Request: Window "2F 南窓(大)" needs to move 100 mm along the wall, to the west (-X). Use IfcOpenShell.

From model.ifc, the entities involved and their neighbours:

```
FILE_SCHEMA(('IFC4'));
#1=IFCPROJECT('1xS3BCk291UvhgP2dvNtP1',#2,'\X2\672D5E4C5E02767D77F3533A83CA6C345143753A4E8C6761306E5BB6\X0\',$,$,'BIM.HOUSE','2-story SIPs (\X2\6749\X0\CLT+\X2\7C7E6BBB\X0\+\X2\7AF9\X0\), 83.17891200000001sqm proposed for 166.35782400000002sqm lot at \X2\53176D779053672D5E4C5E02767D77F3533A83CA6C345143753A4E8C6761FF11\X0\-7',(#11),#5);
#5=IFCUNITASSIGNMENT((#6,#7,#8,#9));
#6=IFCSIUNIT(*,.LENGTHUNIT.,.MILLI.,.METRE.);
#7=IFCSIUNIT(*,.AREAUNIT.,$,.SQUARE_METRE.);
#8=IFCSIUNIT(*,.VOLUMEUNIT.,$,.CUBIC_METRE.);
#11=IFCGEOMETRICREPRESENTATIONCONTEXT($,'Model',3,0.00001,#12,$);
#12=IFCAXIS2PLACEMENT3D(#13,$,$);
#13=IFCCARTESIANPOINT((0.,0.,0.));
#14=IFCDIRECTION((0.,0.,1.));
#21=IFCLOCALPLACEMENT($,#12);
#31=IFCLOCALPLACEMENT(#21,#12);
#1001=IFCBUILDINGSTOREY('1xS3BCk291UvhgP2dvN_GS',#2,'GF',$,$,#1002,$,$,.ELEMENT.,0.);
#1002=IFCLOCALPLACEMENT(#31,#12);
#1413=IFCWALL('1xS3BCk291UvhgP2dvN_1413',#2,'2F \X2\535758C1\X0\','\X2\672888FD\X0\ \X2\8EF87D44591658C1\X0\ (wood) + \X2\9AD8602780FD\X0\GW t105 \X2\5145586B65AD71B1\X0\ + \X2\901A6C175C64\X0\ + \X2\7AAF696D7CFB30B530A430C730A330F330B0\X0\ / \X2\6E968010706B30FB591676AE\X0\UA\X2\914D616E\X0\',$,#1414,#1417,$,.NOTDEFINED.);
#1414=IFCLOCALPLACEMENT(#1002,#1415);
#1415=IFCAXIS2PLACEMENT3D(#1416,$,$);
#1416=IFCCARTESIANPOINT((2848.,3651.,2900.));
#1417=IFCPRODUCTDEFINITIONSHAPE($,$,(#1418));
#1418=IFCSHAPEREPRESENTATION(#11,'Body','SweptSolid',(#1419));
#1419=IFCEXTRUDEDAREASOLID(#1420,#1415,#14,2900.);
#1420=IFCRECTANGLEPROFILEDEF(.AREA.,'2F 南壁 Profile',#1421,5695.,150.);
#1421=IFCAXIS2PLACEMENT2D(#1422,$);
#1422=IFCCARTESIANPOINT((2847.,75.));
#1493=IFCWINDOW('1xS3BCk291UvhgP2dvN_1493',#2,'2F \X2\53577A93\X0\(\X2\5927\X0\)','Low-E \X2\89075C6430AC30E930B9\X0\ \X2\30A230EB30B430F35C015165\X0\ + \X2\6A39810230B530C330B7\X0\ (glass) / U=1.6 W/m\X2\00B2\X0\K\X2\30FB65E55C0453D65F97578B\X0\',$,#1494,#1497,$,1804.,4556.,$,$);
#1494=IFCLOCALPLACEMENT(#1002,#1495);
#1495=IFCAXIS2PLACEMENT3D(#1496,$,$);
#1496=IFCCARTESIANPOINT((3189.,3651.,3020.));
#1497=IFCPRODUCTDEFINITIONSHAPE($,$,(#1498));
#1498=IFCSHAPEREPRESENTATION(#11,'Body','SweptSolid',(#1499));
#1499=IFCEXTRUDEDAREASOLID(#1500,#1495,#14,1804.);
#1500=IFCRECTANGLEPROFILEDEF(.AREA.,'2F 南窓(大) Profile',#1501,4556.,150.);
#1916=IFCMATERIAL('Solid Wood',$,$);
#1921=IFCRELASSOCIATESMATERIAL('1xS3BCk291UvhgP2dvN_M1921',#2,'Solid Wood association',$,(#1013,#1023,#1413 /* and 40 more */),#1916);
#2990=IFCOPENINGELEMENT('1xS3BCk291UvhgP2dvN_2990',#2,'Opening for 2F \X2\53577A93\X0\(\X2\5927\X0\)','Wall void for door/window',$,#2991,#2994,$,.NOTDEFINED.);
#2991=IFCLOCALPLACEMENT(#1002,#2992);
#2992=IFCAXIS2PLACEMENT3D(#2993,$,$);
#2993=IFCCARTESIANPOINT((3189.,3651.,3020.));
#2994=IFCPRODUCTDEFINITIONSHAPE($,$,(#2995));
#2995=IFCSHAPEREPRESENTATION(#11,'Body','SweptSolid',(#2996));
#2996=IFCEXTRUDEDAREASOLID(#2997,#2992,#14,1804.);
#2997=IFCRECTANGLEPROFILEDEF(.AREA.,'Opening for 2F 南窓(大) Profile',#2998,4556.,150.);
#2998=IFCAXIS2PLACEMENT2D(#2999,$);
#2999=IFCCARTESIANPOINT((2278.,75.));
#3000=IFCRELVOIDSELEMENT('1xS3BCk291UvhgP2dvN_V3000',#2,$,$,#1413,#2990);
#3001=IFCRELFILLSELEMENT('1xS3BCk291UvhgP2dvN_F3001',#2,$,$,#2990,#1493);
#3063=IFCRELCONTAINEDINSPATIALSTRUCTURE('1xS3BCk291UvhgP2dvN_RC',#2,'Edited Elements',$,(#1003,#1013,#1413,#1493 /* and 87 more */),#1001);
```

```python
import ifcopenshell
import ifcopenshell.api.geometry
import ifcopenshell.util.placement

model = ifcopenshell.open("model.ifc")

window = model.by_guid("1xS3BCk291UvhgP2dvN_1493")
opening = window.FillsVoids[0].RelatingOpeningElement
wall = opening.VoidsElements[0].RelatingBuildingElement

wall_matrix = ifcopenshell.util.placement.get_local_placement(wall.ObjectPlacement)
shift = wall_matrix[:3, 0] * -100.0
before = ifcopenshell.util.placement.get_local_placement(window.ObjectPlacement)[:3, 3].copy()

# The window is not placed relative to its opening, so move both.
for product in (opening, window):
    matrix = ifcopenshell.util.placement.get_local_placement(product.ObjectPlacement)
    matrix[:3, 3] += shift
    ifcopenshell.api.geometry.edit_object_placement(model, product=product, matrix=matrix, is_si=False)

after = ifcopenshell.util.placement.get_local_placement(window.ObjectPlacement)[:3, 3]
print("window moved by", (after - before).round(3) + 0.0)

model.write("model_rev.ifc")
```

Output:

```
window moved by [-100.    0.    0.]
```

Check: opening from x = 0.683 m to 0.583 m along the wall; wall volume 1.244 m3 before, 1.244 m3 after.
